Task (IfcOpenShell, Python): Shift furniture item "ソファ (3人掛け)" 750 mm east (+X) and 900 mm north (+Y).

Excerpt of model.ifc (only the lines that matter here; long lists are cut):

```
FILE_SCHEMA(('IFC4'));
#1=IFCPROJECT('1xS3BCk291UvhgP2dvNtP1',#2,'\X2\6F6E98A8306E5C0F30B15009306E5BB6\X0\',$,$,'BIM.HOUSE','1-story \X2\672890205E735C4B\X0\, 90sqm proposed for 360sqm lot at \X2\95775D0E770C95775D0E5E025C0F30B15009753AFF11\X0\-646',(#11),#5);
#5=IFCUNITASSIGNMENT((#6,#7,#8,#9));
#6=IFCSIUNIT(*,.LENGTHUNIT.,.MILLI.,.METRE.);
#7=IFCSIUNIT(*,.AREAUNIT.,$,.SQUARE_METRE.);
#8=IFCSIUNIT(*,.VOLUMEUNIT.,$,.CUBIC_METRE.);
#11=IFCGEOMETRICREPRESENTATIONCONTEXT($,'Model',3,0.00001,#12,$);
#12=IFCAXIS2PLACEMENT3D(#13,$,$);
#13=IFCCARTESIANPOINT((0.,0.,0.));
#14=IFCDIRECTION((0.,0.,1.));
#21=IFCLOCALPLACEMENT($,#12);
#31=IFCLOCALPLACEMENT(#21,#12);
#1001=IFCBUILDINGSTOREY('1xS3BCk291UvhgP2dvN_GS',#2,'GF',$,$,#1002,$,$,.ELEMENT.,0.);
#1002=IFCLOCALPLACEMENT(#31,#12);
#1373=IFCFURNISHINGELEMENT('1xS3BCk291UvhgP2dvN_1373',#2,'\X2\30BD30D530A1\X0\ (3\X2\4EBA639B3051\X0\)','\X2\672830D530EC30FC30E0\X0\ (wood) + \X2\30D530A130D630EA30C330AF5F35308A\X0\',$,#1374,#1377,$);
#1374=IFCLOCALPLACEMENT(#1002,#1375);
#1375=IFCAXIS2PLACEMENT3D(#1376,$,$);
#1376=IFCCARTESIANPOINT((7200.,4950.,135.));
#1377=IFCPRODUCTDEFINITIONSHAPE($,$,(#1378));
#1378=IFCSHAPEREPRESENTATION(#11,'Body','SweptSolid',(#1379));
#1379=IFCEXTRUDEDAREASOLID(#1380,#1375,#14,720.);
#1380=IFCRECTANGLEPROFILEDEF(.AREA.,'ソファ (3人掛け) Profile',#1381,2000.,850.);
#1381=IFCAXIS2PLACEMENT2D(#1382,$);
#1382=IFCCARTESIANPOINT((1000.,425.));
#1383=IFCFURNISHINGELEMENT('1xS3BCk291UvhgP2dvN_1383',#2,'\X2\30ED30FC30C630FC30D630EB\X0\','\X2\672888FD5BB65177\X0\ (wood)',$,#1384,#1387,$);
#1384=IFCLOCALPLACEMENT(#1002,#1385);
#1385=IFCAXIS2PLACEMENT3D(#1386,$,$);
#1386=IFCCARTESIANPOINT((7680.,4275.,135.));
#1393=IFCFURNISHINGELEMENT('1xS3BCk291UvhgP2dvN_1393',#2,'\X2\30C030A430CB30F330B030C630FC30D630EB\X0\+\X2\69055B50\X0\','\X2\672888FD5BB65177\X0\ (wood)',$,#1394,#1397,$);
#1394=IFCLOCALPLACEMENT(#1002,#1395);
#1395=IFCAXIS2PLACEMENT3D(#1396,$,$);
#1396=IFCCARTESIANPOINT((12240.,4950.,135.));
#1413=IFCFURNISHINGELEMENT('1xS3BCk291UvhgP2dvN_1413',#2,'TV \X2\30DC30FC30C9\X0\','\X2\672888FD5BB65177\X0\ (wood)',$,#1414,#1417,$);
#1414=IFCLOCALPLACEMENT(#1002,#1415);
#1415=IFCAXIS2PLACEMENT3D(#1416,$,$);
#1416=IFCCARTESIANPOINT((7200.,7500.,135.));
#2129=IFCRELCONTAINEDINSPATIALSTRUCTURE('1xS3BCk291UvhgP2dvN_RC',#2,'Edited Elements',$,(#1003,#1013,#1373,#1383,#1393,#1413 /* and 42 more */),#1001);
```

```python
import ifcopenshell
import ifcopenshell.api.geometry
import ifcopenshell.util.placement
import ifcopenshell.util.unit

model = ifcopenshell.open("model.ifc")
unit_scale = ifcopenshell.util.unit.calculate_unit_scale(model)

item = model.by_guid("1xS3BCk291UvhgP2dvN_1373")
matrix = ifcopenshell.util.placement.get_local_placement(item.ObjectPlacement)
matrix[0, 3] += 0.75 / unit_scale
matrix[1, 3] += 0.9 / unit_scale
ifcopenshell.api.geometry.edit_object_placement(model, product=item, matrix=matrix, is_si=False)

print(ifcopenshell.util.placement.get_local_placement(item.ObjectPlacement).round(3) + 0.0)

model.write("model-out.ifc")
```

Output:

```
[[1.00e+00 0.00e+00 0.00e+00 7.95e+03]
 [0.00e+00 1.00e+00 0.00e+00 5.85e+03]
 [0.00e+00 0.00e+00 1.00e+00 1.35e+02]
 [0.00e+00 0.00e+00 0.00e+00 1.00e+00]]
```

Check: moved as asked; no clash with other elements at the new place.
